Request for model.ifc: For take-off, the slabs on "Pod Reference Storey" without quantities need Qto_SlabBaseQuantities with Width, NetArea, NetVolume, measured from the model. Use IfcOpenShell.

First a look at what the model holds.

```python
import ifcopenshell
import ifcopenshell.util.element
import ifcopenshell.util.unit

model = ifcopenshell.open("model.ifc")
print(model.schema)
for unit_type in ("LENGTHUNIT", "AREAUNIT", "VOLUMEUNIT"):
    print(unit_type, ifcopenshell.util.unit.calculate_unit_scale(model, unit_type))
storey = next(s for s in model.by_type("IfcBuildingStorey") if s.Name == "Pod Reference Storey")
slabs = [e for e in ifcopenshell.util.element.get_decomposition(storey) if e.is_a("IfcSlab")]
for e in sorted(slabs, key=lambda e: e.id()):
    print(e.id(), e.is_a(), e.Name, list(ifcopenshell.util.element.get_psets(e, qtos_only=True)), sep=" | ")
```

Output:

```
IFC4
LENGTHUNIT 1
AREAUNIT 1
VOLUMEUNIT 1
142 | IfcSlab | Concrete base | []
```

```python
import ifcopenshell
import ifcopenshell.api.pset
import ifcopenshell.geom
import ifcopenshell.util.element
import ifcopenshell.util.shape
import ifcopenshell.util.unit

model = ifcopenshell.open("model.ifc")
unit_scale = ifcopenshell.util.unit.calculate_unit_scale(model)
area_scale = ifcopenshell.util.unit.calculate_unit_scale(model, "AREAUNIT")
volume_scale = ifcopenshell.util.unit.calculate_unit_scale(model, "VOLUMEUNIT")
settings = ifcopenshell.geom.settings()

storey = next(s for s in model.by_type("IfcBuildingStorey") if s.Name == "Pod Reference Storey")
slabs = [e for e in ifcopenshell.util.element.get_decomposition(storey) if e.is_a("IfcSlab")]

for e in sorted(slabs, key=lambda e: e.id()):
    if ifcopenshell.util.element.get_psets(e, qtos_only=True, should_inherit=False):
        continue
    # Geometry comes back in metres, in the element's own axes.
    shape = ifcopenshell.geom.create_shape(settings, e)
    values = {
        "Width": ifcopenshell.util.shape.get_z(shape.geometry) / unit_scale,
        "NetArea": ifcopenshell.util.shape.get_footprint_area(shape.geometry) / area_scale,
        "NetVolume": ifcopenshell.util.shape.get_volume(shape.geometry) / volume_scale,
    }
    qto = ifcopenshell.api.pset.add_qto(model, product=e, name="Qto_SlabBaseQuantities")
    ifcopenshell.api.pset.edit_qto(model, qto=qto, properties=values)
    print(e.id(), {k: round(v, 3) for k, v in values.items()})

model.write("model-out.ifc")
```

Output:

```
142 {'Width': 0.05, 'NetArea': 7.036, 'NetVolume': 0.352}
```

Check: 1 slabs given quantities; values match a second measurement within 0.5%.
